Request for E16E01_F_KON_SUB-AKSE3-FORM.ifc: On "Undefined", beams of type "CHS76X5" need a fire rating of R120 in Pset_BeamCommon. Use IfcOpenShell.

First a look at what the model holds.

```python
import ifcopenshell
import ifcopenshell.util.element

model = ifcopenshell.open("E16E01_F_KON_SUB-AKSE3-FORM.ifc")
print(model.schema)
storey = next(s for s in model.by_type("IfcBuildingStorey") if s.Name == "Undefined")
beams = [e for e in ifcopenshell.util.element.get_decomposition(storey) if e.is_a("IfcBeam")]
seen = {}
for e in beams:
    element_type = ifcopenshell.util.element.get_type(e)
    key = (element_type.Name if element_type != e and element_type else None, ifcopenshell.util.element.get_pset(e, "Pset_BeamCommon", "FireRating"))
    seen[key] = seen.get(key, 0) + 1
for (name, value), count in sorted(seen.items(), key=str):
    print(count, "x", name, "|", value)
```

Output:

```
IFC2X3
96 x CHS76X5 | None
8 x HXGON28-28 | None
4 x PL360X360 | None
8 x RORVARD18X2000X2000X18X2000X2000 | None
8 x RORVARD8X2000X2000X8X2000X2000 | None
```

```python
import ifcopenshell
import ifcopenshell.api.pset
import ifcopenshell.util.element

model = ifcopenshell.open("E16E01_F_KON_SUB-AKSE3-FORM.ifc")

storey = next(s for s in model.by_type("IfcBuildingStorey") if s.Name == "Undefined")
beams = [e for e in ifcopenshell.util.element.get_decomposition(storey) if e.is_a("IfcBeam")]

count = 0
for e in beams:
    element_type = ifcopenshell.util.element.get_type(e)
    if element_type in (None, e) or element_type.Name != "CHS76X5":
        continue
    found = ifcopenshell.util.element.get_pset(e, "Pset_BeamCommon", should_inherit=False)
    if found:
        pset = model.by_id(found["id"])
        if len(ifcopenshell.util.element.get_elements_by_pset(pset)) > 1:
            pset = ifcopenshell.api.pset.unshare_pset(model, products=[e], pset=pset)[0]
    else:
        pset = ifcopenshell.api.pset.add_pset(model, product=e, name="Pset_BeamCommon")
    ifcopenshell.api.pset.edit_pset(model, pset=pset, properties={"FireRating": "R120"})
    count += 1

print(count, "beams updated")

model.write("E16E01_F_KON_SUB-AKSE3-FORM-out.ifc")
```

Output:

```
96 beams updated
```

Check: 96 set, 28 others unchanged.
